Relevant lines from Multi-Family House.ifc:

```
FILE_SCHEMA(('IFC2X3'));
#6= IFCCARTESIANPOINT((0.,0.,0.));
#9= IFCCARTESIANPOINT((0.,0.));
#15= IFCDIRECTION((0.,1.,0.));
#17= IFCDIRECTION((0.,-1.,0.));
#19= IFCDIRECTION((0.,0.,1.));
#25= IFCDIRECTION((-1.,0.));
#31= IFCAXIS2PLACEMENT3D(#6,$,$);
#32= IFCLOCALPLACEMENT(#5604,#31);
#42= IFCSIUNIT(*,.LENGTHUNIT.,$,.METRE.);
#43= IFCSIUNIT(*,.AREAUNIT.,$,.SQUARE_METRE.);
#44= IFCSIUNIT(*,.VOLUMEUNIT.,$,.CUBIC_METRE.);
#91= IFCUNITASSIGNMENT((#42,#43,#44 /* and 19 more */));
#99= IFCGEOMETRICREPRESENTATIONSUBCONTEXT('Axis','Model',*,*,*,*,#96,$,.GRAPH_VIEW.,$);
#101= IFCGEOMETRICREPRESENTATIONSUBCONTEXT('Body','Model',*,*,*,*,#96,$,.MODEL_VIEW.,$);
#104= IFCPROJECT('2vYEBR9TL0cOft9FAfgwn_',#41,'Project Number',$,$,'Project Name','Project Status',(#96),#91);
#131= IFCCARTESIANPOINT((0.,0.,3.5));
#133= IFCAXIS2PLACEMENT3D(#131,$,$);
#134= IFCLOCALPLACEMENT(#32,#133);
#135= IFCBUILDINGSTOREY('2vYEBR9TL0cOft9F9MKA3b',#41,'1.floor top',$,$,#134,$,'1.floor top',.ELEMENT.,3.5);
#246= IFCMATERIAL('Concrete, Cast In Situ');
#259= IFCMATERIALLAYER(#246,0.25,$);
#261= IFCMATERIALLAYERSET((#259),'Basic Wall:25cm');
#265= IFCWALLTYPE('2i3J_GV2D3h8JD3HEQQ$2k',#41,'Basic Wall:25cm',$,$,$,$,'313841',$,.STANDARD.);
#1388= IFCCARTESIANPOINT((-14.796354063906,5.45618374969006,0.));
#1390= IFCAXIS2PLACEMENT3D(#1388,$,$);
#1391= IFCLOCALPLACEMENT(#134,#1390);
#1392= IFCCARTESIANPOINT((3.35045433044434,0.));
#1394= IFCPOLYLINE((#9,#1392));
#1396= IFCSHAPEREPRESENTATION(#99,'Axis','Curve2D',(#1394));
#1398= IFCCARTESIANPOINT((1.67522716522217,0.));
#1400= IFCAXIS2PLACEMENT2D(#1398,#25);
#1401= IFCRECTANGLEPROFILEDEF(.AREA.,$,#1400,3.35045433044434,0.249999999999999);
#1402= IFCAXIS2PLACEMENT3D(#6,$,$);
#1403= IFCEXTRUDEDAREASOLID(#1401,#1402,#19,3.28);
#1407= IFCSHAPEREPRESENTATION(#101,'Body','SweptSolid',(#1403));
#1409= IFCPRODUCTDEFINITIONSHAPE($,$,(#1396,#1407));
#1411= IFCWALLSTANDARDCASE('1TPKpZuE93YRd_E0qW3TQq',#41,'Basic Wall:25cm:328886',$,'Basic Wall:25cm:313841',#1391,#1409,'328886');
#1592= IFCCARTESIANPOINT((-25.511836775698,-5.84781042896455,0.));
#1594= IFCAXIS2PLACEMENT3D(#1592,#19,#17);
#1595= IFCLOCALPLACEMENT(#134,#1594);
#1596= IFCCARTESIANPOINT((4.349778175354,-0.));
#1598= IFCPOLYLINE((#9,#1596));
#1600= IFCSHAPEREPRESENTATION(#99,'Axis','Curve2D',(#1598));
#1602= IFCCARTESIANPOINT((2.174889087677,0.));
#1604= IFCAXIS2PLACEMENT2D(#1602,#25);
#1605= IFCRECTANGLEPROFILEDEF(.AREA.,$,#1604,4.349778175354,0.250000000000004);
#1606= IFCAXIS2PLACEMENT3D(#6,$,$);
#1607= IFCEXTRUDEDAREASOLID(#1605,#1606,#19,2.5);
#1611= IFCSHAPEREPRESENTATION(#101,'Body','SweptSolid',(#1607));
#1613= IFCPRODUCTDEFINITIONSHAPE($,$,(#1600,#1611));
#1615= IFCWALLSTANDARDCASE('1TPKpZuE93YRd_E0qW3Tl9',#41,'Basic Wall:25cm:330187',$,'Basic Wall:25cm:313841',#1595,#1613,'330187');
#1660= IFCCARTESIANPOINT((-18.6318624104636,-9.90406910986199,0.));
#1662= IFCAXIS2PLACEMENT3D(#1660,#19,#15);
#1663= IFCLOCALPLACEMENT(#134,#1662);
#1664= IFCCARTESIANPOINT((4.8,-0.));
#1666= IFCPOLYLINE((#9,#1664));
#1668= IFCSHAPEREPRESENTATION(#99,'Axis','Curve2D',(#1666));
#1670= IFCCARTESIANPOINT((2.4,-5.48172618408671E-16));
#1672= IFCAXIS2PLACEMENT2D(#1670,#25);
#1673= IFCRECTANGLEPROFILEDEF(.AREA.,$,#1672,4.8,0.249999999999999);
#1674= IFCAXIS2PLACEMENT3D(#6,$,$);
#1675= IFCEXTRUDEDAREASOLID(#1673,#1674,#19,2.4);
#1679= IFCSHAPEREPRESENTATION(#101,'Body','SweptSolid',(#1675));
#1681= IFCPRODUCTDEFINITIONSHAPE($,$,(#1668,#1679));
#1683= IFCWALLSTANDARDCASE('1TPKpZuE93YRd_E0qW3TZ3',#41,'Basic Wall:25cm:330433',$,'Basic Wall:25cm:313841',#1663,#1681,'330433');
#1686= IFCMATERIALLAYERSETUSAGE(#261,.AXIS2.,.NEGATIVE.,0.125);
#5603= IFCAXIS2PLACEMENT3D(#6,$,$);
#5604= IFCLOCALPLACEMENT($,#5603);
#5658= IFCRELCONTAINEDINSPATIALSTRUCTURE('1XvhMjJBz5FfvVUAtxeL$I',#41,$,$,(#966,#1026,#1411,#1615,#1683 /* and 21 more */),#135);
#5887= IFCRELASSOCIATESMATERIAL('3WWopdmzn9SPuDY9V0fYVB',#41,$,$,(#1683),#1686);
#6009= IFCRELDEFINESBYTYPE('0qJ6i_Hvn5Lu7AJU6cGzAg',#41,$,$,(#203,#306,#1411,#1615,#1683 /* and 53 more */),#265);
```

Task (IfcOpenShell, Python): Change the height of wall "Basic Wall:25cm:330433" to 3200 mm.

```python
import ifcopenshell
import ifcopenshell.geom
import ifcopenshell.util.representation
import ifcopenshell.util.shape

model = ifcopenshell.open("Multi-Family House.ifc")
settings = ifcopenshell.geom.settings()


def volume(element):
    """Net volume in cubic metres, openings subtracted."""
    shape = ifcopenshell.geom.create_shape(settings, element)
    return ifcopenshell.util.shape.get_volume(shape.geometry)


wall = model.by_id(1683)
before = volume(wall)

body = ifcopenshell.util.representation.get_representation(wall, "Model", "Body")
solid = body.Items[0]
old_height = solid.Depth
solid.Depth = 3.2
after = volume(wall)

print(f"height {old_height:g} -> {solid.Depth:g}, volume {before:.3f} -> {after:.3f} m3")

model.write("Multi-Family House_v2.ifc")
```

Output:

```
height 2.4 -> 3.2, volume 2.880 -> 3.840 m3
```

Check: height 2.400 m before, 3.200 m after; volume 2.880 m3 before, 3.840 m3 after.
